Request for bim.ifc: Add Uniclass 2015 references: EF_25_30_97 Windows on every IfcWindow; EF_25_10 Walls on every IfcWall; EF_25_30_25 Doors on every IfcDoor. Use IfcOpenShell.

First a look at what the model holds.

```python
import ifcopenshell

model = ifcopenshell.open("bim.ifc")
print(model.schema)
print("classifications:", [c.Name for c in model.by_type("IfcClassification")])
for ifc_class in ("IfcDoor", "IfcRoof", "IfcStair", "IfcWall", "IfcWindow"):
    print(ifc_class, len(model.by_type(ifc_class)))
```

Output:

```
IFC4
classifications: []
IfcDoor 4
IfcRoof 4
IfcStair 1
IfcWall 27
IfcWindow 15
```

```python
import ifcopenshell
import ifcopenshell.api.classification

model = ifcopenshell.open("bim.ifc")

system = ifcopenshell.api.classification.add_classification(model, classification="Uniclass 2015")

codes = {
    "IfcWindow": ("EF_25_30_97", "Windows"),
    "IfcWall": ("EF_25_10", "Walls"),
    "IfcDoor": ("EF_25_30_25", "Doors"),
}
for ifc_class, (code, name) in codes.items():
    products = model.by_type(ifc_class)
    ifcopenshell.api.classification.add_reference(
        model, products=products, classification=system, identification=code, name=name
    )
    print(code, len(products))

model.write("bim_rev.ifc")
```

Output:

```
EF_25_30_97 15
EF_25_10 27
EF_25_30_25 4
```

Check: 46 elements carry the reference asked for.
